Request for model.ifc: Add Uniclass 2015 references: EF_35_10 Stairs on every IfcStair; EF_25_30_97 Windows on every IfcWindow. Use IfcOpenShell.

First a look at what the model holds.

```python
import ifcopenshell

model = ifcopenshell.open("model.ifc")
print(model.schema)
print("classifications:", [c.Name for c in model.by_type("IfcClassification")])
for ifc_class in ("IfcDoor", "IfcRoof", "IfcStair", "IfcWall", "IfcWindow"):
    print(ifc_class, len(model.by_type(ifc_class)))
```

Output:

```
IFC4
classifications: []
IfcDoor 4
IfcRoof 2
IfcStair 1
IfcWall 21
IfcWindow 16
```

```python
import ifcopenshell
import ifcopenshell.api.classification

model = ifcopenshell.open("model.ifc")

system = ifcopenshell.api.classification.add_classification(model, classification="Uniclass 2015")

codes = {
    "IfcStair": ("EF_35_10", "Stairs"),
    "IfcWindow": ("EF_25_30_97", "Windows"),
}
for ifc_class, (code, name) in codes.items():
    products = model.by_type(ifc_class)
    ifcopenshell.api.classification.add_reference(
        model, products=products, classification=system, identification=code, name=name
    )
    print(code, len(products))

model.write("model-out.ifc")
```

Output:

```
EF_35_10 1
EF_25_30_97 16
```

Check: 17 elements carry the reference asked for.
